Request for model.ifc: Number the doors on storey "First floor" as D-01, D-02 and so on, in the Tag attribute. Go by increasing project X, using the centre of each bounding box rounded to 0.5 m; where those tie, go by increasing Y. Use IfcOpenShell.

First a look at what the model holds.

```python
import ifcopenshell
import ifcopenshell.util.element
import ifcopenshell.util.placement

model = ifcopenshell.open("model.ifc")
print(model.schema)
storey = next(s for s in model.by_type("IfcBuildingStorey") if s.Name == "First floor")
doors = [e for e in ifcopenshell.util.element.get_decomposition(storey) if e.is_a("IfcDoor")]
for e in sorted(doors, key=lambda e: e.id()):
    origin = ifcopenshell.util.placement.get_local_placement(e.ObjectPlacement)[:3, 3]
    print(e.id(), e.Tag, e.Name, origin.round(2) + 0.0, sep=" | ")
```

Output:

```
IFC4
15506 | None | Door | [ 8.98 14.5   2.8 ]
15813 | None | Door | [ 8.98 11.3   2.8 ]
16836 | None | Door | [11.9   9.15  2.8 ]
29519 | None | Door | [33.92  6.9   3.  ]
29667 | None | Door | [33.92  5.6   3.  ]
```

```python
import ifcopenshell
import ifcopenshell.geom
import ifcopenshell.util.element
import ifcopenshell.util.shape

model = ifcopenshell.open("model.ifc")
settings = ifcopenshell.geom.settings()
settings.set("use-world-coords", True)


def centre(element):
    shape = ifcopenshell.geom.create_shape(settings, element)
    return ifcopenshell.util.shape.get_bbox_centroid(shape.geometry)


storey = next(s for s in model.by_type("IfcBuildingStorey") if s.Name == "First floor")
doors = [e for e in ifcopenshell.util.element.get_decomposition(storey) if e.is_a("IfcDoor")]

# Insertion points can sit at a corner or the storey origin, so sort by the geometry (in metres).
centres = {e: centre(e) for e in doors}
doors.sort(key=lambda e: (round(centres[e][0] / 0.5), centres[e][1]))

for i, e in enumerate(doors, start=1):
    number = f"D-{i:02d}"
    e.Tag = number
    print(e.id(), number)

model.write("model_rev.ifc")
```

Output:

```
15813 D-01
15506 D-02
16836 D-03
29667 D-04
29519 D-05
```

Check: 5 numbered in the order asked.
